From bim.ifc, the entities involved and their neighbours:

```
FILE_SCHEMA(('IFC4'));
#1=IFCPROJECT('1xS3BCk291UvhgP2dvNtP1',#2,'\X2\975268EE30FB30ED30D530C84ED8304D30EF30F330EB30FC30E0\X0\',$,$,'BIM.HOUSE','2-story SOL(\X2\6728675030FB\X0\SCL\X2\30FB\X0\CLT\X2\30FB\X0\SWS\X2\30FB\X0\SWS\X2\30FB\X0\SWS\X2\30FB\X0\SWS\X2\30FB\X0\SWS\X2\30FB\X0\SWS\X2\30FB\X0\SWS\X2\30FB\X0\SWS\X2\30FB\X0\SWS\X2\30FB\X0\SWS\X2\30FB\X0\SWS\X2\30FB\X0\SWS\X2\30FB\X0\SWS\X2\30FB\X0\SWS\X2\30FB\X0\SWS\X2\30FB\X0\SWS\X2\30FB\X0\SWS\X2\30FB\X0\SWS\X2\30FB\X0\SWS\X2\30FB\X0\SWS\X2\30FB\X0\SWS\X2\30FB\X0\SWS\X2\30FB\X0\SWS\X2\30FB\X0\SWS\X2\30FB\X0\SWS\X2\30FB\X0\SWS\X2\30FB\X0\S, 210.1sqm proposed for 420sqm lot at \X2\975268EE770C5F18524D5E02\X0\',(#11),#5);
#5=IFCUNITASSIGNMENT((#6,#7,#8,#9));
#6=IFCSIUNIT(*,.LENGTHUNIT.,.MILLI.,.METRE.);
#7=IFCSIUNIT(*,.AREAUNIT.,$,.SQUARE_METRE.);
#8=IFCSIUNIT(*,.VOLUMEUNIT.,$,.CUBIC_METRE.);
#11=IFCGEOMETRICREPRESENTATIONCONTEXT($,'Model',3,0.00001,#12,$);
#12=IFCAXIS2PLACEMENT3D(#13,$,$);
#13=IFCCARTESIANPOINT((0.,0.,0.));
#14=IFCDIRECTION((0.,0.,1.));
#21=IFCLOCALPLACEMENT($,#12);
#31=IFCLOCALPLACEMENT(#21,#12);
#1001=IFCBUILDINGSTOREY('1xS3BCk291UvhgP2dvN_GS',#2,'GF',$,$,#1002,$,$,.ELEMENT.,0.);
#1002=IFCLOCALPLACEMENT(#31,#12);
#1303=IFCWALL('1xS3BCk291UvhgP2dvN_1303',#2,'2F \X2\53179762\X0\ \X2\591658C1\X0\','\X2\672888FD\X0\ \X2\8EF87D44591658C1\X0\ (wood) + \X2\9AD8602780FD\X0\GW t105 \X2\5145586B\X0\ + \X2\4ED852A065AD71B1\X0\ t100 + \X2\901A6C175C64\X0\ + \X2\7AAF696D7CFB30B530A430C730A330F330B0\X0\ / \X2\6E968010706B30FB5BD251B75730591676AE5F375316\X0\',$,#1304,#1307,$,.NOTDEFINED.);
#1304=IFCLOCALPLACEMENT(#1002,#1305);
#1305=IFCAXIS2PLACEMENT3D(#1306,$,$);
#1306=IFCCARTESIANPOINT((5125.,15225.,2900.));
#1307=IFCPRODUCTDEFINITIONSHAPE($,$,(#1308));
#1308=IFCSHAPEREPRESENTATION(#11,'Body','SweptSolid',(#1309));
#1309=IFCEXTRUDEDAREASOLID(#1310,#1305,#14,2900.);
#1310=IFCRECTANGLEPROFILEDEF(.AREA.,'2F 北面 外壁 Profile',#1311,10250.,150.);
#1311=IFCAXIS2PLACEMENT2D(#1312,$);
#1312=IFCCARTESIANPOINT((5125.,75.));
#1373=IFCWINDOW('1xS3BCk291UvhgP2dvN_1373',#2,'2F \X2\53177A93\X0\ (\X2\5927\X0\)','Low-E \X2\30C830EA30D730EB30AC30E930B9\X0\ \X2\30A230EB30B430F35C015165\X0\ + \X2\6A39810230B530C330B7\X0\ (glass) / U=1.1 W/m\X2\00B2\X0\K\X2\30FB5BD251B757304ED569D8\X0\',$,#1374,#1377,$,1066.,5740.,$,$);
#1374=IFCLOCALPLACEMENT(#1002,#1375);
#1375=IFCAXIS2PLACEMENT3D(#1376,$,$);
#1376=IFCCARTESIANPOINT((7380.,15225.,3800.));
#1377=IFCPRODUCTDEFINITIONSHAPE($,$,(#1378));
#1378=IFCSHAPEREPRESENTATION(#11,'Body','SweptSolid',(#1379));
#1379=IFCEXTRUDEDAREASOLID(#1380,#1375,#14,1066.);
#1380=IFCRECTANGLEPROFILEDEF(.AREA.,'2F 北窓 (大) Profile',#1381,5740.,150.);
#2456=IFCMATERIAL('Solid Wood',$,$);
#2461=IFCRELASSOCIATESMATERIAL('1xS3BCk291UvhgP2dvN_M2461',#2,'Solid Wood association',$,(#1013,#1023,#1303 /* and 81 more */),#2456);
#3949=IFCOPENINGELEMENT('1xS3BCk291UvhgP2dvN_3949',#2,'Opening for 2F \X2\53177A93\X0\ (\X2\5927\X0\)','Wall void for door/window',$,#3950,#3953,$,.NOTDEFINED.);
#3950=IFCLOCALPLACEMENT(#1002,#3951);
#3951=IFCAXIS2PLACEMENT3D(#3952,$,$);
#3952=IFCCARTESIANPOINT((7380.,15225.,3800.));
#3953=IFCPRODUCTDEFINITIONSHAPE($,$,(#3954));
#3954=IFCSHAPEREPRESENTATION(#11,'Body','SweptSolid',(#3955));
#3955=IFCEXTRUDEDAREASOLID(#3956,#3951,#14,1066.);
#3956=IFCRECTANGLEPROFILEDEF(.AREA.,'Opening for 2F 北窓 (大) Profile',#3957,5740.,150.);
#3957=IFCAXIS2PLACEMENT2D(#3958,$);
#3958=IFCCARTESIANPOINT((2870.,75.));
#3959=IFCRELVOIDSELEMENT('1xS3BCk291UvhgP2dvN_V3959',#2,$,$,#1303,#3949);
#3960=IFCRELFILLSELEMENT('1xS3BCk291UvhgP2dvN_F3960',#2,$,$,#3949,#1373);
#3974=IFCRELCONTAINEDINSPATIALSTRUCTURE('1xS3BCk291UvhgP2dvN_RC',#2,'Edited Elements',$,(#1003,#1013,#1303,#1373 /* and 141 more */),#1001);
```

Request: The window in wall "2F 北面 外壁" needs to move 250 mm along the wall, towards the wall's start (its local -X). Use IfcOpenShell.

```python
import ifcopenshell
import ifcopenshell.api.geometry
import ifcopenshell.util.placement
import ifcopenshell.util.unit

model = ifcopenshell.open("bim.ifc")
unit_scale = ifcopenshell.util.unit.calculate_unit_scale(model)

window = model.by_id(1373)
opening = window.FillsVoids[0].RelatingOpeningElement
wall = opening.VoidsElements[0].RelatingBuildingElement

wall_matrix = ifcopenshell.util.placement.get_local_placement(wall.ObjectPlacement)
shift = wall_matrix[:3, 0] * -0.25 / unit_scale
before = ifcopenshell.util.placement.get_local_placement(window.ObjectPlacement)[:3, 3].copy()

# The window is not placed relative to its opening, so move both.
for product in (opening, window):
    matrix = ifcopenshell.util.placement.get_local_placement(product.ObjectPlacement)
    matrix[:3, 3] += shift
    ifcopenshell.api.geometry.edit_object_placement(model, product=product, matrix=matrix, is_si=False)

after = ifcopenshell.util.placement.get_local_placement(window.ObjectPlacement)[:3, 3]
print("window moved by", (after - before).round(3) + 0.0)

model.write("bim-out.ifc")
```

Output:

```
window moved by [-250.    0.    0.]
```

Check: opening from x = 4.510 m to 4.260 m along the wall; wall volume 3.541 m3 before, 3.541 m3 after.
